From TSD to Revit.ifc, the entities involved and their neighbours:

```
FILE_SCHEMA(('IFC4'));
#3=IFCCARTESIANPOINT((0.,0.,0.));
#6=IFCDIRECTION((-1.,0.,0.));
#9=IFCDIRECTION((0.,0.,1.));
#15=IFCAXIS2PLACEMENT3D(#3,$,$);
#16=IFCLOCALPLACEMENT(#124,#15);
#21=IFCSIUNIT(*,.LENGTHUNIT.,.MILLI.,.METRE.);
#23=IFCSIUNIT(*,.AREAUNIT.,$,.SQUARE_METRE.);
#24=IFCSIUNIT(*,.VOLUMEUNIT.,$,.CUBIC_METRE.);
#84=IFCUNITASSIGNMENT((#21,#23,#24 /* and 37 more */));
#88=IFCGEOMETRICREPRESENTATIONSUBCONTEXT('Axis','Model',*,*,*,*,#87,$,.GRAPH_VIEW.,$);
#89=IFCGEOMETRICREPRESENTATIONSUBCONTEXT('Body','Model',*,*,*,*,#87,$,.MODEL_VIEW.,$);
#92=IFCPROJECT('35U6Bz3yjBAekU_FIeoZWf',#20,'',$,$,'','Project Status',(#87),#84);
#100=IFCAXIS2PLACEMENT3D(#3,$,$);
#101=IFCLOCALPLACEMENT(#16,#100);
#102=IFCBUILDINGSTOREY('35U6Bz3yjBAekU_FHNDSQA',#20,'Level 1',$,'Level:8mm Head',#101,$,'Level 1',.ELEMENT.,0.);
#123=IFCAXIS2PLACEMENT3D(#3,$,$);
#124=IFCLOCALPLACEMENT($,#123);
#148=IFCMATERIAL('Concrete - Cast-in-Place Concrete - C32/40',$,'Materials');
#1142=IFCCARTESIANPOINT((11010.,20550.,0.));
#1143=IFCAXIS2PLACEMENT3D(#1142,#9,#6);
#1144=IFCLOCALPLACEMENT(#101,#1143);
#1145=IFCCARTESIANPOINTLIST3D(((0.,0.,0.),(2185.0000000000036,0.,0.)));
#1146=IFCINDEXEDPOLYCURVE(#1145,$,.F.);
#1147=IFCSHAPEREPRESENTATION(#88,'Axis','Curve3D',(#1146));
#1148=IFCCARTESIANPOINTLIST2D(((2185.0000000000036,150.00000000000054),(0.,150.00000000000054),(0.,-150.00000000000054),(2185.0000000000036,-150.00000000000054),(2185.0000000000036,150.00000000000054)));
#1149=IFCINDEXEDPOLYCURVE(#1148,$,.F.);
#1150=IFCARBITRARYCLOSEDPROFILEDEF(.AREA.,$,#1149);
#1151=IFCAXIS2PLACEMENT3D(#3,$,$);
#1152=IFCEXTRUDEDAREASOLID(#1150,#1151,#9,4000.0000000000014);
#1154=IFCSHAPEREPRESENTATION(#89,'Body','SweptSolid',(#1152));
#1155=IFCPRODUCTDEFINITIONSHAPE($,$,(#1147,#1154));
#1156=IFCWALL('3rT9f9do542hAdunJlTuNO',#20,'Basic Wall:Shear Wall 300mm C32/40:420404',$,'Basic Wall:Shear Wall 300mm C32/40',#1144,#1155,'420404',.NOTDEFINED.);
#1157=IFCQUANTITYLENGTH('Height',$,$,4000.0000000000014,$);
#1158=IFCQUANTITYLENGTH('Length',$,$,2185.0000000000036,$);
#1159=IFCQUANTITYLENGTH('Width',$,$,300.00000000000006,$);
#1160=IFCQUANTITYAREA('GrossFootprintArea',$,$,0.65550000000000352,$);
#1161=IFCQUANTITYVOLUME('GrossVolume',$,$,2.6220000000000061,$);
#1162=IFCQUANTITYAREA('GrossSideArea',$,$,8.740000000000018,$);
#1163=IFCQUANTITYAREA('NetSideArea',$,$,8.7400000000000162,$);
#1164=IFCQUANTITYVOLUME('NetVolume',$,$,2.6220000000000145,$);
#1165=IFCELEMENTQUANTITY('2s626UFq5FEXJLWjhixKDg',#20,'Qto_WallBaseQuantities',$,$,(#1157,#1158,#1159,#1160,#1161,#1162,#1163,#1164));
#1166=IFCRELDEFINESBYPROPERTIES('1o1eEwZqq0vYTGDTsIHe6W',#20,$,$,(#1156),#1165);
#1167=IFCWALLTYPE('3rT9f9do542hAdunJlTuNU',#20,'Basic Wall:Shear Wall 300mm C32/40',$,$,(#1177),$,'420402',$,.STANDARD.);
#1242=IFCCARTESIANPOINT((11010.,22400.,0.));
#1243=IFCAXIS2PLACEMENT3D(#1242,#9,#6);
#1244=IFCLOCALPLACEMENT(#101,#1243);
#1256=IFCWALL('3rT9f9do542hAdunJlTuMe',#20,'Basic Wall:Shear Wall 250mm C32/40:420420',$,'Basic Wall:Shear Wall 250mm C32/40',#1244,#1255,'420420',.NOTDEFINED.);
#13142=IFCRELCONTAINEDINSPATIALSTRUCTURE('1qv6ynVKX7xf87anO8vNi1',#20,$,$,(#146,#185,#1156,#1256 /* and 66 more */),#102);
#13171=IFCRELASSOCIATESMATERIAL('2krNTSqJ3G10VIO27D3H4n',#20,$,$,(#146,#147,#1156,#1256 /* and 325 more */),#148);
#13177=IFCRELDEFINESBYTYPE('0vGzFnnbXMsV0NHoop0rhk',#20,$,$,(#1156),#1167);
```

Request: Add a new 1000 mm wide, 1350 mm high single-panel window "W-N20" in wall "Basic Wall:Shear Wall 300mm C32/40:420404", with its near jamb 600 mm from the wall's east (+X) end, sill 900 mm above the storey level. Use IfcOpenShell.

```python
import numpy as np
import ifcopenshell
import ifcopenshell.api.feature
import ifcopenshell.api.geometry
import ifcopenshell.api.pset
import ifcopenshell.api.root
import ifcopenshell.api.spatial
import ifcopenshell.geom
import ifcopenshell.util.element
import ifcopenshell.util.placement
import ifcopenshell.util.representation
import ifcopenshell.util.shape
import ifcopenshell.util.unit

model = ifcopenshell.open("TSD to Revit.ifc")
unit_scale = ifcopenshell.util.unit.calculate_unit_scale(model)
area_scale = ifcopenshell.util.unit.calculate_unit_scale(model, "AREAUNIT")
volume_scale = ifcopenshell.util.unit.calculate_unit_scale(model, "VOLUMEUNIT")
settings = ifcopenshell.geom.settings()


def volume(element):
    """Net volume in cubic metres, openings subtracted."""
    shape = ifcopenshell.geom.create_shape(settings, element)
    return ifcopenshell.util.shape.get_volume(shape.geometry)


wall = model.by_guid("3rT9f9do542hAdunJlTuNO")
storey = ifcopenshell.util.element.get_container(wall, ifc_class="IfcBuildingStorey")
context = ifcopenshell.util.representation.get_context(model, "Model", "Body", "MODEL_VIEW")
before = volume(wall)

width, height, from_end, sill = 1, 1.35, 0.6, 0.9  # metres

# The wall runs along its own X axis, and the end named is its -X end.
wall_shape = ifcopenshell.geom.create_shape(settings, wall)
x, y, z = ifcopenshell.util.shape.get_vertices(wall_shape.geometry).T
start = x.min() + from_end
face, thickness = float(y.min()), float(y.max() - y.min())
wall_matrix = ifcopenshell.util.placement.get_local_placement(wall.ObjectPlacement)
level = ifcopenshell.util.placement.get_local_placement(storey.ObjectPlacement)[2, 3]


def in_wall(x, y):
    """Placement at x, y metres in the wall's axes, at sill height."""
    matrix = wall_matrix.copy()
    matrix[:, 3] = wall_matrix @ np.array([x / unit_scale, y / unit_scale, 0.0, 1.0])
    matrix[2, 3] = level + sill / unit_scale
    return matrix


# Opening: a box that overshoots both wall faces by 50 mm.
opening = ifcopenshell.api.root.create_entity(model, ifc_class="IfcOpeningElement", predefined_type="OPENING")
box = ifcopenshell.api.geometry.add_wall_representation(
    model, context=context, length=width, height=height, thickness=thickness + 0.1
)
ifcopenshell.api.geometry.assign_representation(model, product=opening, representation=box)
ifcopenshell.api.geometry.edit_object_placement(model, product=opening, matrix=in_wall(start, face - 0.05), is_si=False)
ifcopenshell.api.feature.add_feature(model, feature=opening, element=wall)

window = ifcopenshell.api.root.create_entity(model, ifc_class="IfcWindow", name="W-N20", predefined_type="WINDOW")
window.OverallWidth, window.OverallHeight = width / unit_scale, height / unit_scale
window.PartitioningType = "SINGLE_PANEL"
body = ifcopenshell.api.geometry.add_window_representation(
    model,
    context=context,
    overall_width=window.OverallWidth,
    overall_height=window.OverallHeight,
    partition_type="SINGLE_PANEL",
)
ifcopenshell.api.geometry.assign_representation(model, product=window, representation=body)
ifcopenshell.api.spatial.assign_container(model, products=[window], relating_structure=storey)
ifcopenshell.api.feature.add_filling(model, opening=opening, element=window)

# Centre the window in the wall's thickness.
ifcopenshell.api.geometry.edit_object_placement(model, product=window, matrix=in_wall(start, face), is_si=False)
window_shape = ifcopenshell.geom.create_shape(settings, window)
depth = ifcopenshell.util.shape.get_vertices(window_shape.geometry)[:, 1]
offset = face + thickness / 2 - (depth.min() + depth.max()) / 2
ifcopenshell.api.geometry.edit_object_placement(model, product=window, matrix=in_wall(start, offset), is_si=False)

after = volume(wall)

# Update the wall's stored quantities.
qto = model.by_id(ifcopenshell.util.element.get_pset(wall, "Qto_WallBaseQuantities", should_inherit=False)["id"])
ifcopenshell.api.pset.edit_qto(model, qto=qto, properties={
    "NetSideArea": after / thickness / area_scale,
    "NetVolume": after / volume_scale,
})

print(f"wall volume {before:.3f} -> {after:.3f} m3")

model.write("TSD to Revit_rev.ifc")
```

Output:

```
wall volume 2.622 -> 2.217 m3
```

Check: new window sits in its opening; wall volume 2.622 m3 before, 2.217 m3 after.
